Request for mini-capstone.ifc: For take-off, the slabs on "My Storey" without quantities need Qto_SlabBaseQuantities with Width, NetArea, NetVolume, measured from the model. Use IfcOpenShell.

First a look at what the model holds.

```python
import ifcopenshell
import ifcopenshell.util.element
import ifcopenshell.util.unit

model = ifcopenshell.open("mini-capstone.ifc")
print(model.schema)
for unit_type in ("LENGTHUNIT", "AREAUNIT", "VOLUMEUNIT"):
    print(unit_type, ifcopenshell.util.unit.calculate_unit_scale(model, unit_type))
storey = next(s for s in model.by_type("IfcBuildingStorey") if s.Name == "My Storey")
slabs = [e for e in ifcopenshell.util.element.get_decomposition(storey) if e.is_a("IfcSlab")]
for e in sorted(slabs, key=lambda e: e.id()):
    print(e.id(), e.is_a(), e.Name, list(ifcopenshell.util.element.get_psets(e, qtos_only=True)), sep=" | ")
```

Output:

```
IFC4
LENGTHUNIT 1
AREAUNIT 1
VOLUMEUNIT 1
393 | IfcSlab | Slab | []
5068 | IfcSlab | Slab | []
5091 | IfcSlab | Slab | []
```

```python
import ifcopenshell
import ifcopenshell.api.pset
import ifcopenshell.geom
import ifcopenshell.util.element
import ifcopenshell.util.shape
import ifcopenshell.util.unit

model = ifcopenshell.open("mini-capstone.ifc")
unit_scale = ifcopenshell.util.unit.calculate_unit_scale(model)
area_scale = ifcopenshell.util.unit.calculate_unit_scale(model, "AREAUNIT")
volume_scale = ifcopenshell.util.unit.calculate_unit_scale(model, "VOLUMEUNIT")
settings = ifcopenshell.geom.settings()

storey = next(s for s in model.by_type("IfcBuildingStorey") if s.Name == "My Storey")
slabs = [e for e in ifcopenshell.util.element.get_decomposition(storey) if e.is_a("IfcSlab")]

for e in sorted(slabs, key=lambda e: e.id()):
    if ifcopenshell.util.element.get_psets(e, qtos_only=True, should_inherit=False):
        continue
    # Geometry comes back in metres, in the element's own axes.
    shape = ifcopenshell.geom.create_shape(settings, e)
    values = {
        "Width": ifcopenshell.util.shape.get_z(shape.geometry) / unit_scale,
        "NetArea": ifcopenshell.util.shape.get_footprint_area(shape.geometry) / area_scale,
        "NetVolume": ifcopenshell.util.shape.get_volume(shape.geometry) / volume_scale,
    }
    qto = ifcopenshell.api.pset.add_qto(model, product=e, name="Qto_SlabBaseQuantities")
    ifcopenshell.api.pset.edit_qto(model, qto=qto, properties=values)
    print(e.id(), {k: round(v, 3) for k, v in values.items()})

model.write("mini-capstone_rev.ifc")
```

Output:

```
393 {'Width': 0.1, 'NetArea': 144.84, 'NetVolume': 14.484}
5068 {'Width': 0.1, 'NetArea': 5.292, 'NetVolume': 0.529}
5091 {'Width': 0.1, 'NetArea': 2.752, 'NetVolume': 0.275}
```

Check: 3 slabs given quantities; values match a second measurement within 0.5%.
